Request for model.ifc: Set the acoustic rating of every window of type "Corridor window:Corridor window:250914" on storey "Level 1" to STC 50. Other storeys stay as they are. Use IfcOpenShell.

First a look at what the model holds.

```python
import ifcopenshell
import ifcopenshell.util.element

model = ifcopenshell.open("model.ifc")
print(model.schema)
storey = next(s for s in model.by_type("IfcBuildingStorey") if s.Name == "Level 1")
windows = [e for e in ifcopenshell.util.element.get_decomposition(storey) if e.is_a("IfcWindow")]
seen = {}
for e in windows:
    element_type = ifcopenshell.util.element.get_type(e)
    key = (element_type.Name if element_type != e and element_type else None, ifcopenshell.util.element.get_pset(e, "Pset_WindowCommon", "AcousticRating"))
    seen[key] = seen.get(key, 0) + 1
for (name, value), count in sorted(seen.items(), key=str):
    print(count, "x", name, "|", value)
```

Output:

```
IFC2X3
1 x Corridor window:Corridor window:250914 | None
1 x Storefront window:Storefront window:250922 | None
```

```python
import ifcopenshell
import ifcopenshell.api.pset
import ifcopenshell.util.element

model = ifcopenshell.open("model.ifc")

storey = next(s for s in model.by_type("IfcBuildingStorey") if s.Name == "Level 1")
windows = [e for e in ifcopenshell.util.element.get_decomposition(storey) if e.is_a("IfcWindow")]

count = 0
for e in windows:
    element_type = ifcopenshell.util.element.get_type(e)
    if element_type in (None, e) or element_type.Name != "Corridor window:Corridor window:250914":
        continue
    # add_pset returns the element's existing set when there is one.
    pset = ifcopenshell.api.pset.add_pset(model, product=e, name="Pset_WindowCommon")
    ifcopenshell.api.pset.edit_pset(model, pset=pset, properties={"AcousticRating": "STC 50"})
    count += 1

print(count, "windows updated")

model.write("model_updated.ifc")
```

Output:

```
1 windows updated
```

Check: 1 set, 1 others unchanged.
